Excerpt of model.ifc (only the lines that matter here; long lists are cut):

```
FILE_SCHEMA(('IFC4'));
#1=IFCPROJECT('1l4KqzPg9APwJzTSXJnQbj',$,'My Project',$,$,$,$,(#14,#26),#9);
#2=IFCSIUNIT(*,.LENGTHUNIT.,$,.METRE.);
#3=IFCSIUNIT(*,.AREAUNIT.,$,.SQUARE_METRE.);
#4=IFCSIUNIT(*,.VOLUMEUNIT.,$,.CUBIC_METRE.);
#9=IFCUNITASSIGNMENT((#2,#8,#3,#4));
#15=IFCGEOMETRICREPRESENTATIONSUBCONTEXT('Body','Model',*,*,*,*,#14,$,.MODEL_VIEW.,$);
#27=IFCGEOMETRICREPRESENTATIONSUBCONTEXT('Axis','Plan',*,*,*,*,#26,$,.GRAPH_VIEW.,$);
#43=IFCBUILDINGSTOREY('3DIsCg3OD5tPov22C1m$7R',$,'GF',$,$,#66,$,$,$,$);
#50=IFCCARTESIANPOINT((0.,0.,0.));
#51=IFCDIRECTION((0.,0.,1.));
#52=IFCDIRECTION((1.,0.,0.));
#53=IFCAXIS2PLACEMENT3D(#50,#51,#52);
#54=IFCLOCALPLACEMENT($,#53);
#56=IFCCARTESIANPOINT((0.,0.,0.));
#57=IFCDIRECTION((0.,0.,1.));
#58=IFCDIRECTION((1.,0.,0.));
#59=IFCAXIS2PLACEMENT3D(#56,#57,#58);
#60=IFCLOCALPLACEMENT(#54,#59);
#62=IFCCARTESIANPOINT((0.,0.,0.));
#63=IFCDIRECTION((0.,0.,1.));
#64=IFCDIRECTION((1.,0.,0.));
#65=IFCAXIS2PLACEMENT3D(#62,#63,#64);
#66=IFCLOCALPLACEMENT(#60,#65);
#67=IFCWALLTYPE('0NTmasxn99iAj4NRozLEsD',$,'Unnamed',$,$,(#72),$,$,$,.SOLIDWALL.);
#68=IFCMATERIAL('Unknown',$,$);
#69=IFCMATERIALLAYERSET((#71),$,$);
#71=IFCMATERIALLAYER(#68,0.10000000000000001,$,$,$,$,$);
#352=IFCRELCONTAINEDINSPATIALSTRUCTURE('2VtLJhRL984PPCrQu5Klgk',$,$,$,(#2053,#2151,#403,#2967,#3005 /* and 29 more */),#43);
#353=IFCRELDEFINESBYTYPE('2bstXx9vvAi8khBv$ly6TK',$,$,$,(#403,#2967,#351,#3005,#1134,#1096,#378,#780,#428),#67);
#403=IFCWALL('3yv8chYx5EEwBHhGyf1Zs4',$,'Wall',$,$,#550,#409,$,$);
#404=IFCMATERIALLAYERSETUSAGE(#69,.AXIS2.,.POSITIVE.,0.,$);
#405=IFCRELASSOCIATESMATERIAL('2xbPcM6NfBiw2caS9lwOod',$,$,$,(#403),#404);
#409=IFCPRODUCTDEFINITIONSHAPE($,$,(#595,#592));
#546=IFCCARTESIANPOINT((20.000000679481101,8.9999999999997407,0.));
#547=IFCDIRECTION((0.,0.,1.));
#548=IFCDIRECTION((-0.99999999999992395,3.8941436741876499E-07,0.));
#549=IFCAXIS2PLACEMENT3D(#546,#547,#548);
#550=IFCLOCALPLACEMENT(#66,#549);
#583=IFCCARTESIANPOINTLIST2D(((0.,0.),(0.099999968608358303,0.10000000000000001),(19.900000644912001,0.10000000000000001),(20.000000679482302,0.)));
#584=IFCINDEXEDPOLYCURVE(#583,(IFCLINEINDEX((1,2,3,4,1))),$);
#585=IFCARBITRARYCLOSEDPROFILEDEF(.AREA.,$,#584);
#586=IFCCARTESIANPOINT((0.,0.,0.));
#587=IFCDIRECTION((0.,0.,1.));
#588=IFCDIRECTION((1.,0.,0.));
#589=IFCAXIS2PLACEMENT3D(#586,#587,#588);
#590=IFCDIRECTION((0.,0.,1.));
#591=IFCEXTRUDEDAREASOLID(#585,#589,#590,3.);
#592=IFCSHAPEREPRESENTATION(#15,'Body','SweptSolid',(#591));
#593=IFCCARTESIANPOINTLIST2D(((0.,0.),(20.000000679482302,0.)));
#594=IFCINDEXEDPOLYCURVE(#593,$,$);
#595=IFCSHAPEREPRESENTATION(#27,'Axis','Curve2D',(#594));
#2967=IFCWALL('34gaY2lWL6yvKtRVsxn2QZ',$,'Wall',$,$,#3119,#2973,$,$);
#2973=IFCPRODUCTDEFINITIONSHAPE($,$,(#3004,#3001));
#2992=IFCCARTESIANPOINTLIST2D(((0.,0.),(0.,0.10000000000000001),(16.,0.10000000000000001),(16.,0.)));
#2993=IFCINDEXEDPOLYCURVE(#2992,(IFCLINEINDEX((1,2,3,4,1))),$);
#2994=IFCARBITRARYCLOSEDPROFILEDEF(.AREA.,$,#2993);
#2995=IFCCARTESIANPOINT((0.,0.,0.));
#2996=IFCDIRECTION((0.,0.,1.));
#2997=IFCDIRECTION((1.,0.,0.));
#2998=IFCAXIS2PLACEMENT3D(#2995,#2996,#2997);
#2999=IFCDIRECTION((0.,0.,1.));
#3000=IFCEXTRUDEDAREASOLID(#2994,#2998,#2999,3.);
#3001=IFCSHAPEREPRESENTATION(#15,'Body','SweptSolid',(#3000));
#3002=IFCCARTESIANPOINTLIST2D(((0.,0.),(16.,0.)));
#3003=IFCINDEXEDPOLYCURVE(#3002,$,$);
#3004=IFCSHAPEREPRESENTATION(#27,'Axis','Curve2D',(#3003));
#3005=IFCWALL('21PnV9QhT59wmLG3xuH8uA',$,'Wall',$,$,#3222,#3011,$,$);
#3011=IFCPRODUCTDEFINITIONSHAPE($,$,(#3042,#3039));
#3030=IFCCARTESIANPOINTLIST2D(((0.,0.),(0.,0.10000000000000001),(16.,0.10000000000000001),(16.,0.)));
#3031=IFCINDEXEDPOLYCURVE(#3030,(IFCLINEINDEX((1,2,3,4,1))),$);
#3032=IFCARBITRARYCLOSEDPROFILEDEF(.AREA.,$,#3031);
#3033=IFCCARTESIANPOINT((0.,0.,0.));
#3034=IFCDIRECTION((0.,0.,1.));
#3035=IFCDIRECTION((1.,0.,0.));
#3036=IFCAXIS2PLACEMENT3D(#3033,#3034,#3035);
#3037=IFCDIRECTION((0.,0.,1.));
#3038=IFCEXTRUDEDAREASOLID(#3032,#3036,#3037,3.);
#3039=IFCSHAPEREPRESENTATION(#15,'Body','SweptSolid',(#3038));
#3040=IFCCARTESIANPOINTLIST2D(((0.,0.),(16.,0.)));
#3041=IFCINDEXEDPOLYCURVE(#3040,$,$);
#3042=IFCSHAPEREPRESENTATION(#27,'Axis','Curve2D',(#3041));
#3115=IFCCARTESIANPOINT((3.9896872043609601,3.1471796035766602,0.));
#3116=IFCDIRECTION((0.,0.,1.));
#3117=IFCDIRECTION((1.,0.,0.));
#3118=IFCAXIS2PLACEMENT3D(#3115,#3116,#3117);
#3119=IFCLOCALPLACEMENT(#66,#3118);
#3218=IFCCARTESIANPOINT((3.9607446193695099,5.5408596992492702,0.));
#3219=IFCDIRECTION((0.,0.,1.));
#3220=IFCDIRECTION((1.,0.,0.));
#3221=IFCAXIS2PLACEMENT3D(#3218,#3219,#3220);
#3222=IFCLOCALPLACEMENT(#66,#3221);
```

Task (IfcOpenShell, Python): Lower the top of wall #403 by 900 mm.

```python
import ifcopenshell
import ifcopenshell.geom
import ifcopenshell.util.representation
import ifcopenshell.util.shape
import ifcopenshell.util.unit

model = ifcopenshell.open("model.ifc")
unit_scale = ifcopenshell.util.unit.calculate_unit_scale(model)
settings = ifcopenshell.geom.settings()


def volume(element):
    """Net volume in cubic metres, openings subtracted."""
    shape = ifcopenshell.geom.create_shape(settings, element)
    return ifcopenshell.util.shape.get_volume(shape.geometry)


wall = model.by_guid("3yv8chYx5EEwBHhGyf1Zs4")
before = volume(wall)

body = ifcopenshell.util.representation.get_representation(wall, "Model", "Body")
solid = body.Items[0]
old_height = solid.Depth
solid.Depth -= 0.9 / unit_scale
after = volume(wall)

print(f"height {old_height:g} -> {solid.Depth:g}, volume {before:.3f} -> {after:.3f} m3")

model.write("model_v2.ifc")
```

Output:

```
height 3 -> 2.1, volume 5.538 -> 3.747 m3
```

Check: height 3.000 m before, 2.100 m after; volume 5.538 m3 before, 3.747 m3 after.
